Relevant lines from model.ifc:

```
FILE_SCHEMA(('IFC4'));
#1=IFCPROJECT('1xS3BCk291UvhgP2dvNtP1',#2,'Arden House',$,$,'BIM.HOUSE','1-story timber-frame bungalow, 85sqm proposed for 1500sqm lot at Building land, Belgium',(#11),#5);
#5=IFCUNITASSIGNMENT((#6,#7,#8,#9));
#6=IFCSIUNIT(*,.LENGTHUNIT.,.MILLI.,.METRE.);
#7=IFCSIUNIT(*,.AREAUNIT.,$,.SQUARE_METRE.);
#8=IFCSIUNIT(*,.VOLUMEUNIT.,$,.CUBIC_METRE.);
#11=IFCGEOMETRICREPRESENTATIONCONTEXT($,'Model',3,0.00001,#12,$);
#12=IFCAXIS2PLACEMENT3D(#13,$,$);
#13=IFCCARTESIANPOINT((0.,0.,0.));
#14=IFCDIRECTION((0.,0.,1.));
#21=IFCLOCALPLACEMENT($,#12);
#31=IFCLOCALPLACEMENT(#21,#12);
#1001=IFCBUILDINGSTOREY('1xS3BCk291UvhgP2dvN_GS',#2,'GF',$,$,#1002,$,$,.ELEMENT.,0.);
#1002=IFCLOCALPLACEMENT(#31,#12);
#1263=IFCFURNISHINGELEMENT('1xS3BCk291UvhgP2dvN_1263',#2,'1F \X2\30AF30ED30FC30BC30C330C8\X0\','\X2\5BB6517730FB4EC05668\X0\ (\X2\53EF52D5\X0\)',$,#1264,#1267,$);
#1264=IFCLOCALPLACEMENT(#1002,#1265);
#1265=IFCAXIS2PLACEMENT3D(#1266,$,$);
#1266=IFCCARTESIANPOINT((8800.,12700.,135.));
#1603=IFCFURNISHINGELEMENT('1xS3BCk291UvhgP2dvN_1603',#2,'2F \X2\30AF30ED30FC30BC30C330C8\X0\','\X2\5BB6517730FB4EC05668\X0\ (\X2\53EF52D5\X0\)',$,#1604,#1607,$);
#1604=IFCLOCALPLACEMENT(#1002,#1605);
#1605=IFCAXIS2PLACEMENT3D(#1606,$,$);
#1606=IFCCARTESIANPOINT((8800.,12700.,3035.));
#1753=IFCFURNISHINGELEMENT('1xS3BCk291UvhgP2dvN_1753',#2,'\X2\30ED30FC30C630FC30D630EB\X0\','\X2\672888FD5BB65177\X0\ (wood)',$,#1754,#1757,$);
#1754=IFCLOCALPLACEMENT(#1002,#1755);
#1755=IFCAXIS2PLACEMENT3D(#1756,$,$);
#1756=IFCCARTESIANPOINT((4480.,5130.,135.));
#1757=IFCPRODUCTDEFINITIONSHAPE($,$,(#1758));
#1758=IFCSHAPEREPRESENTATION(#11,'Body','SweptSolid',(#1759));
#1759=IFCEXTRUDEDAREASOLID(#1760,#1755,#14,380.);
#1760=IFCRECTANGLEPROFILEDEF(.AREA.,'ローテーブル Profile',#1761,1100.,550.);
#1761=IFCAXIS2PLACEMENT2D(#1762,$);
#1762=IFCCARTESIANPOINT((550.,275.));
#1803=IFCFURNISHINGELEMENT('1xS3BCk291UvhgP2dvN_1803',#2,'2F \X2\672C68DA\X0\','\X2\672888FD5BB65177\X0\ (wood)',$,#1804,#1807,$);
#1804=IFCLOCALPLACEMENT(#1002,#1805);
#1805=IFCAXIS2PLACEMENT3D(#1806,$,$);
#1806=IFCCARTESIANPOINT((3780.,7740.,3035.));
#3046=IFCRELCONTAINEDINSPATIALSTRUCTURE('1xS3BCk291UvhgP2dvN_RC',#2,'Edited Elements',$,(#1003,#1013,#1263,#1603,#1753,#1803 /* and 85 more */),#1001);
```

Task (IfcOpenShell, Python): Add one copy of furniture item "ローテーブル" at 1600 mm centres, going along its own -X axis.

```python
import ifcopenshell
import ifcopenshell.api.geometry
import ifcopenshell.api.root
import ifcopenshell.util.element
import ifcopenshell.util.placement
import ifcopenshell.util.unit

model = ifcopenshell.open("model.ifc")
unit_scale = ifcopenshell.util.unit.calculate_unit_scale(model)


def reuse_history(source, copy):
    """copy_class also copies each property set's owner history, people and application; keep the originals."""
    for rel in copy.IsDefinedBy:
        if rel.is_a("IfcRelDefinesByProperties") and (history := rel.RelatingPropertyDefinition.OwnerHistory):
            rel.RelatingPropertyDefinition.OwnerHistory = source.OwnerHistory
            ifcopenshell.util.element.remove_deep2(model, history)


source = model.by_guid("1xS3BCk291UvhgP2dvN_1753")
base = ifcopenshell.util.placement.get_local_placement(source.ObjectPlacement)
step = -base[:3, 0] * 1.6 / unit_scale

for i in range(1, 2):
    copy = ifcopenshell.api.root.copy_class(model, product=source)
    copy.Representation = ifcopenshell.util.element.copy_deep(
        model, source.Representation, exclude=["IfcGeometricRepresentationContext", "IfcRepresentationMap"]
    )
    reuse_history(source, copy)
    matrix = base.copy()
    matrix[:3, 3] += i * step
    print("added at", matrix[:3, 3].round(3) + 0.0)
    ifcopenshell.api.geometry.edit_object_placement(model, product=copy, matrix=matrix, is_si=False)

model.write("model_rev.ifc")
```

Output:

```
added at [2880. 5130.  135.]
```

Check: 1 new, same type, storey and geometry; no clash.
